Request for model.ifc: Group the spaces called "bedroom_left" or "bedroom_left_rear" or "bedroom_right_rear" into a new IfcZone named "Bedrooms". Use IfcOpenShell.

First a look at what the model holds.

```python
import ifcopenshell

model = ifcopenshell.open("model.ifc")
print(model.schema)
seen = {}
for space in model.by_type("IfcSpace"):
    seen[space.LongName] = seen.get(space.LongName, 0) + 1
for name, count in sorted(seen.items(), key=str):
    print(count, "x", name)
print("zones:", [z.Name for z in model.by_type("IfcZone")][:20])
```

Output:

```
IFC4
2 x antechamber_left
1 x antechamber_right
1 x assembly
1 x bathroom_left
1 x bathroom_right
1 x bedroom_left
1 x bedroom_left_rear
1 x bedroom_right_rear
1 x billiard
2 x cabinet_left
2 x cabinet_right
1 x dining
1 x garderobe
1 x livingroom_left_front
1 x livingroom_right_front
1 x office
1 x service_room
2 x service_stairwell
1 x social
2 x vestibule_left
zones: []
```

```python
import ifcopenshell
import ifcopenshell.api.group
import ifcopenshell.api.root

model = ifcopenshell.open("model.ifc")

names = {"bedroom_left", "bedroom_left_rear", "bedroom_right_rear"}
spaces = [s for s in model.by_type("IfcSpace") if s.LongName in names]

zone = ifcopenshell.api.root.create_entity(model, ifc_class="IfcZone", name="Bedrooms")
ifcopenshell.api.group.assign_group(model, products=spaces, group=zone)
print(len(spaces), "spaces in", zone.Name)

model.write("model_updated.ifc")
```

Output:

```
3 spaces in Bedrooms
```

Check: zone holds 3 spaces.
